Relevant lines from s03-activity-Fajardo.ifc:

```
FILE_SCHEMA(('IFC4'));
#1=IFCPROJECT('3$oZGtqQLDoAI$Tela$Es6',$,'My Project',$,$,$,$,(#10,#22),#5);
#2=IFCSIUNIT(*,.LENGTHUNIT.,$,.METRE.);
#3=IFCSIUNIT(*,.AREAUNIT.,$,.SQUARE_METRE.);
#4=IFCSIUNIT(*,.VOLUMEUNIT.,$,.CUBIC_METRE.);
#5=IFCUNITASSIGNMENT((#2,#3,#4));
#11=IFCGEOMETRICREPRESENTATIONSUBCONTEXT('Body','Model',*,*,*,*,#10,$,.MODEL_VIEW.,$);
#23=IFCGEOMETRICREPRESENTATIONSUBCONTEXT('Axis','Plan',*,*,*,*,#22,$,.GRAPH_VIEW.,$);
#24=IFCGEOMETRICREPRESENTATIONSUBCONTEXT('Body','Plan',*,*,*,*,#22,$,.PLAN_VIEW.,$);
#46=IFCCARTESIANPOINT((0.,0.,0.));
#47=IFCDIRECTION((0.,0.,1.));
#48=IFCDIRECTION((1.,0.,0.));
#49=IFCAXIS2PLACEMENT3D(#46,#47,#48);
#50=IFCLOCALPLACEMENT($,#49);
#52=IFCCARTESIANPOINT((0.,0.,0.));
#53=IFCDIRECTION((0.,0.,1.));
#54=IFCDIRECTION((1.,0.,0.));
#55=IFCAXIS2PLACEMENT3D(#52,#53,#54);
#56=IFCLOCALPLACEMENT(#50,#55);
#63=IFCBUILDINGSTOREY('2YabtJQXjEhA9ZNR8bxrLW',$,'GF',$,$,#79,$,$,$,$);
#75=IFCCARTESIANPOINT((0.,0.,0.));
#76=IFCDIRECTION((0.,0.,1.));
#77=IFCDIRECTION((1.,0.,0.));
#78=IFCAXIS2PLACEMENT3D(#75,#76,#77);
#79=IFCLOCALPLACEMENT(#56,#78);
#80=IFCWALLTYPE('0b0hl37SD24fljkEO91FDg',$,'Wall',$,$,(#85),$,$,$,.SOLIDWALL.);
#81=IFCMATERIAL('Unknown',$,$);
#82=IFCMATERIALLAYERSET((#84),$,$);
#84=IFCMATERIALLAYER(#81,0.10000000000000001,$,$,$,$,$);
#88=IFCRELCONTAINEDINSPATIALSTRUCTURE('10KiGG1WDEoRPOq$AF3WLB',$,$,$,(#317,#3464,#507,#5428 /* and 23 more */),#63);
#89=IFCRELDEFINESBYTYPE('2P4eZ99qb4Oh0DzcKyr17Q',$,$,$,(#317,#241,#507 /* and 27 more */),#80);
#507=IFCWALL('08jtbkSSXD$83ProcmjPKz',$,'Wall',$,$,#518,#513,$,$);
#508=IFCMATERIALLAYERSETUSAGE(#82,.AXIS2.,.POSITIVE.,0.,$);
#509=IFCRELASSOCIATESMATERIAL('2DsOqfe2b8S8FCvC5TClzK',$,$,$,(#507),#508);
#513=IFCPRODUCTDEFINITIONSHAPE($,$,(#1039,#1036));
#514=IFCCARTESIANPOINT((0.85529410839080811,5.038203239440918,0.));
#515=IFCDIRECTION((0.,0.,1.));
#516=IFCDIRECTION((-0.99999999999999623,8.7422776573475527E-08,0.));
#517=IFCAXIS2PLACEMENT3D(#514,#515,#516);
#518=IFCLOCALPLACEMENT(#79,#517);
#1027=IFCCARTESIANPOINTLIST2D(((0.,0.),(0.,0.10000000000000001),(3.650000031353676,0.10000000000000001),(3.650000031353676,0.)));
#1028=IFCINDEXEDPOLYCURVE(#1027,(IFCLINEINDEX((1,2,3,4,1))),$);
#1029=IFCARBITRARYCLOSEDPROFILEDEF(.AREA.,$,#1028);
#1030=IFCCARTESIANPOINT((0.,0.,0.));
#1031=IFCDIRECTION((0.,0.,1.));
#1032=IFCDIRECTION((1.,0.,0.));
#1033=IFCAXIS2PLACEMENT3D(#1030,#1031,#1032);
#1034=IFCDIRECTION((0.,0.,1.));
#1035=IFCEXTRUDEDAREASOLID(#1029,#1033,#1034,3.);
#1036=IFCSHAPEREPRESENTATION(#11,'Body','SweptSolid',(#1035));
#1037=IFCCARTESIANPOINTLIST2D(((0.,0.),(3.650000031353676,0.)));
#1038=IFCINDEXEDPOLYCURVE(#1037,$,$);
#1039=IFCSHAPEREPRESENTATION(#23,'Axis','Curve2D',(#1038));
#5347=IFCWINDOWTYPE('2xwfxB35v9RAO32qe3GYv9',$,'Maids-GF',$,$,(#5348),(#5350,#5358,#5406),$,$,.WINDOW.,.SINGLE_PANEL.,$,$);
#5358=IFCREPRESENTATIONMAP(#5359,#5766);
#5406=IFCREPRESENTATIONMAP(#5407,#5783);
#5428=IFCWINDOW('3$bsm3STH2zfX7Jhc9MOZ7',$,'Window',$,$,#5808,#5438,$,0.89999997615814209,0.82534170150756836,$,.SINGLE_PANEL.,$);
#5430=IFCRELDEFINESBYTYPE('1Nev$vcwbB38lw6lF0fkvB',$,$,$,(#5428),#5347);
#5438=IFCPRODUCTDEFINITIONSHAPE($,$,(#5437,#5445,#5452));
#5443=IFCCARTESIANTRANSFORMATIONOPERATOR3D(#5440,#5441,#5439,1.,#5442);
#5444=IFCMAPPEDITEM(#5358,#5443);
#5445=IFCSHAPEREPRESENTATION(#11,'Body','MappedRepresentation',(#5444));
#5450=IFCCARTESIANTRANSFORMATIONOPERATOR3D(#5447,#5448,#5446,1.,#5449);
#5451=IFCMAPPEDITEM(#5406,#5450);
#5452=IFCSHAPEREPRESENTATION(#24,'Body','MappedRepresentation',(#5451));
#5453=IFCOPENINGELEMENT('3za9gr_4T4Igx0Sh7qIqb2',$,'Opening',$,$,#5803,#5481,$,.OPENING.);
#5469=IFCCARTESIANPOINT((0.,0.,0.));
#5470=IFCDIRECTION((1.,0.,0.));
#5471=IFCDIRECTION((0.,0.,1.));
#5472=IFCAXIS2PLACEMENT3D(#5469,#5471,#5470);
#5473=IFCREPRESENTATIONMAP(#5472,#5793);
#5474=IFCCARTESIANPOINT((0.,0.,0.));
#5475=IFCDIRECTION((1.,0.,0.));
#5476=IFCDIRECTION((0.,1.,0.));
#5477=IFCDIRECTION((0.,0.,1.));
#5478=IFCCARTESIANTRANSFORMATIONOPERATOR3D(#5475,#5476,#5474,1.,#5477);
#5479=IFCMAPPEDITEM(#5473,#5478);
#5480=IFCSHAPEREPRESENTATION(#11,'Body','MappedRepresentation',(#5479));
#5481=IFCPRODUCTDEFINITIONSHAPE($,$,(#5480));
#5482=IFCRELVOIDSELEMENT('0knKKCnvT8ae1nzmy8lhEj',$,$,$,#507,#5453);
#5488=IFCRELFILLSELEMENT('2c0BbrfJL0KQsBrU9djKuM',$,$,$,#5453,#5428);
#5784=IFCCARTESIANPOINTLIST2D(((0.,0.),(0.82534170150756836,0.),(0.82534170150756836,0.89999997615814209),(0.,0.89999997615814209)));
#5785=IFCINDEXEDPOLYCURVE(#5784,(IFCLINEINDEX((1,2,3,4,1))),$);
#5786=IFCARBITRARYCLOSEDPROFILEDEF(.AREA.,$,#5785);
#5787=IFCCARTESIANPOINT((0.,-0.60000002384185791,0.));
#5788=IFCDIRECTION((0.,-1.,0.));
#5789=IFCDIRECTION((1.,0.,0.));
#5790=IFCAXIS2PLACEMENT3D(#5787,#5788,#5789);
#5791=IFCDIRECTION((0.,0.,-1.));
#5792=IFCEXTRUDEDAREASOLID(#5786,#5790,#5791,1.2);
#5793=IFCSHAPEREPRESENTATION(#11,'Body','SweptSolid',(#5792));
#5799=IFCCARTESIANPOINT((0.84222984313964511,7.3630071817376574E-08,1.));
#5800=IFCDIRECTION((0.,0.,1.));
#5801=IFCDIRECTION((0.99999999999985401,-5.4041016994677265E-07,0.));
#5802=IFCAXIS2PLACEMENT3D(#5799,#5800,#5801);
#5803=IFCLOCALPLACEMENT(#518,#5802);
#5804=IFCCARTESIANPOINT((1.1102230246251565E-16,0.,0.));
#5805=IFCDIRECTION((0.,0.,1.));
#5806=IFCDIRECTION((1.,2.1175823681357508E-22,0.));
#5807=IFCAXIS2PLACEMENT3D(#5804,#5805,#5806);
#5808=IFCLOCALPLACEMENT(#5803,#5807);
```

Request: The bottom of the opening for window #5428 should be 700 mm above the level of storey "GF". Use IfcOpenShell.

```python
import numpy as np
import ifcopenshell
import ifcopenshell.api.geometry
import ifcopenshell.geom
import ifcopenshell.util.element
import ifcopenshell.util.placement
import ifcopenshell.util.shape
import ifcopenshell.util.unit

model = ifcopenshell.open("s03-activity-Fajardo.ifc")
unit_scale = ifcopenshell.util.unit.calculate_unit_scale(model)

window = model.by_guid("3$bsm3STH2zfX7Jhc9MOZ7")
opening = window.FillsVoids[0].RelatingOpeningElement
storey = ifcopenshell.util.element.get_container(window, ifc_class="IfcBuildingStorey")
level = ifcopenshell.util.placement.get_local_placement(storey.ObjectPlacement)[2, 3]

# The opening's origin need not be at the sill, so measure its lowest point.
shape = ifcopenshell.geom.create_shape(ifcopenshell.geom.settings(), opening)
bottom = ifcopenshell.util.shape.get_shape_bottom_elevation(shape, shape.geometry) / unit_scale
dz = level + 0.7 / unit_scale - bottom

shift = np.array([0.0, 0.0, dz])
# The window is placed relative to its opening, so it follows when the opening moves.
matrix = ifcopenshell.util.placement.get_local_placement(opening.ObjectPlacement)
matrix[:3, 3] += shift
ifcopenshell.api.geometry.edit_object_placement(
    model, product=opening, matrix=matrix, is_si=False, should_transform_children=True
)

print(f"moved by {dz * unit_scale:+.3f} m")

model.write("s03-activity-Fajardo_edited.ifc")
```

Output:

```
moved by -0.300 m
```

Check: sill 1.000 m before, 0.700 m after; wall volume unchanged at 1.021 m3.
